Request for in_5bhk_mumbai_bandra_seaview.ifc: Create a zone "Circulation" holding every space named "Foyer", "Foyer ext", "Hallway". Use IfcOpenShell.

First a look at what the model holds.

```python
import ifcopenshell

model = ifcopenshell.open("in_5bhk_mumbai_bandra_seaview.ifc")
print(model.schema)
seen = {}
for space in model.by_type("IfcSpace"):
    seen[space.LongName] = seen.get(space.LongName, 0) + 1
for name, count in sorted(seen.items(), key=str):
    print(count, "x", name)
print("zones:", [z.Name for z in model.by_type("IfcZone")][:20])
```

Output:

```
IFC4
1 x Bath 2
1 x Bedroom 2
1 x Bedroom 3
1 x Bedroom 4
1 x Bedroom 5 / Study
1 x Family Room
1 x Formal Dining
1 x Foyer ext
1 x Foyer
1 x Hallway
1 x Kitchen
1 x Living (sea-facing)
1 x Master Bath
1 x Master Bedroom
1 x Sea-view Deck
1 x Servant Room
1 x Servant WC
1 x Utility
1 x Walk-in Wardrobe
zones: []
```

```python
import ifcopenshell
import ifcopenshell.api.group
import ifcopenshell.api.root

model = ifcopenshell.open("in_5bhk_mumbai_bandra_seaview.ifc")

names = {"Foyer", "Foyer ext", "Hallway"}
spaces = [s for s in model.by_type("IfcSpace") if s.LongName in names]

zone = ifcopenshell.api.root.create_entity(model, ifc_class="IfcZone", name="Circulation")
ifcopenshell.api.group.assign_group(model, products=spaces, group=zone)
print(len(spaces), "spaces in", zone.Name)

model.write("in_5bhk_mumbai_bandra_seaview_v2.ifc")
```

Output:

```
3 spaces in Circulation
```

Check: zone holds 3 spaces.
